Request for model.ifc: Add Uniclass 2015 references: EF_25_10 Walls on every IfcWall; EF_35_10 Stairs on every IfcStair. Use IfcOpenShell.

First a look at what the model holds.

```python
import ifcopenshell

model = ifcopenshell.open("model.ifc")
print(model.schema)
print("classifications:", [c.Name for c in model.by_type("IfcClassification")])
for ifc_class in ("IfcDoor", "IfcRoof", "IfcStair", "IfcWall", "IfcWindow"):
    print(ifc_class, len(model.by_type(ifc_class)))
```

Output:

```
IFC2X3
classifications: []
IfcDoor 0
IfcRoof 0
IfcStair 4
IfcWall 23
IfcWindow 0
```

```python
import ifcopenshell
import ifcopenshell.api.classification

model = ifcopenshell.open("model.ifc")

# IFC2X3 requires Source and Edition and has no link from the project to the system.
system = model.create_entity("IfcClassification", Source="NBS", Edition="2015", Name="Uniclass 2015")

codes = {
    "IfcWall": ("EF_25_10", "Walls"),
    "IfcStair": ("EF_35_10", "Stairs"),
}
for ifc_class, (code, name) in codes.items():
    products = model.by_type(ifc_class)
    ifcopenshell.api.classification.add_reference(
        model, products=products, classification=system, identification=code, name=name
    )
    print(code, len(products))

model.write("model_rev.ifc")
```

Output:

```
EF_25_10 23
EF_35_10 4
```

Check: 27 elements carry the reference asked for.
